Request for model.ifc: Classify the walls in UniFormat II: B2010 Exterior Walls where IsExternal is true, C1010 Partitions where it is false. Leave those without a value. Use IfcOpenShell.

First a look at what the model holds.

```python
import ifcopenshell
import ifcopenshell.util.element

model = ifcopenshell.open("model.ifc")
print(model.schema)
print("classifications:", [c.Name for c in model.by_type("IfcClassification")])
values = [ifcopenshell.util.element.get_pset(e, "Pset_WallCommon", "IsExternal") for e in model.by_type("IfcWall")]
for value in (True, False, None):
    print("IsExternal", value, values.count(value))
```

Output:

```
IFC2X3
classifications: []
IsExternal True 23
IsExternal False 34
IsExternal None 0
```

```python
import ifcopenshell
import ifcopenshell.api.classification
import ifcopenshell.util.element

model = ifcopenshell.open("model.ifc")

# IFC2X3 requires Source and Edition and has no link from the project to the system.
system = model.create_entity("IfcClassification", Source="ASTM", Edition="E1557", Name="UniFormat II")

walls = model.by_type("IfcWall")
external = {e: ifcopenshell.util.element.get_pset(e, "Pset_WallCommon", "IsExternal") for e in walls}
for flag, code, name in ((True, "B2010", "Exterior Walls"), (False, "C1010", "Partitions")):
    products = [e for e in walls if external[e] is flag]
    ifcopenshell.api.classification.add_reference(
        model, products=products, classification=system, identification=code, name=name
    )
    print(code, len(products))

model.write("model_edited.ifc")
```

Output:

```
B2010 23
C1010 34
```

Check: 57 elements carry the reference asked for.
